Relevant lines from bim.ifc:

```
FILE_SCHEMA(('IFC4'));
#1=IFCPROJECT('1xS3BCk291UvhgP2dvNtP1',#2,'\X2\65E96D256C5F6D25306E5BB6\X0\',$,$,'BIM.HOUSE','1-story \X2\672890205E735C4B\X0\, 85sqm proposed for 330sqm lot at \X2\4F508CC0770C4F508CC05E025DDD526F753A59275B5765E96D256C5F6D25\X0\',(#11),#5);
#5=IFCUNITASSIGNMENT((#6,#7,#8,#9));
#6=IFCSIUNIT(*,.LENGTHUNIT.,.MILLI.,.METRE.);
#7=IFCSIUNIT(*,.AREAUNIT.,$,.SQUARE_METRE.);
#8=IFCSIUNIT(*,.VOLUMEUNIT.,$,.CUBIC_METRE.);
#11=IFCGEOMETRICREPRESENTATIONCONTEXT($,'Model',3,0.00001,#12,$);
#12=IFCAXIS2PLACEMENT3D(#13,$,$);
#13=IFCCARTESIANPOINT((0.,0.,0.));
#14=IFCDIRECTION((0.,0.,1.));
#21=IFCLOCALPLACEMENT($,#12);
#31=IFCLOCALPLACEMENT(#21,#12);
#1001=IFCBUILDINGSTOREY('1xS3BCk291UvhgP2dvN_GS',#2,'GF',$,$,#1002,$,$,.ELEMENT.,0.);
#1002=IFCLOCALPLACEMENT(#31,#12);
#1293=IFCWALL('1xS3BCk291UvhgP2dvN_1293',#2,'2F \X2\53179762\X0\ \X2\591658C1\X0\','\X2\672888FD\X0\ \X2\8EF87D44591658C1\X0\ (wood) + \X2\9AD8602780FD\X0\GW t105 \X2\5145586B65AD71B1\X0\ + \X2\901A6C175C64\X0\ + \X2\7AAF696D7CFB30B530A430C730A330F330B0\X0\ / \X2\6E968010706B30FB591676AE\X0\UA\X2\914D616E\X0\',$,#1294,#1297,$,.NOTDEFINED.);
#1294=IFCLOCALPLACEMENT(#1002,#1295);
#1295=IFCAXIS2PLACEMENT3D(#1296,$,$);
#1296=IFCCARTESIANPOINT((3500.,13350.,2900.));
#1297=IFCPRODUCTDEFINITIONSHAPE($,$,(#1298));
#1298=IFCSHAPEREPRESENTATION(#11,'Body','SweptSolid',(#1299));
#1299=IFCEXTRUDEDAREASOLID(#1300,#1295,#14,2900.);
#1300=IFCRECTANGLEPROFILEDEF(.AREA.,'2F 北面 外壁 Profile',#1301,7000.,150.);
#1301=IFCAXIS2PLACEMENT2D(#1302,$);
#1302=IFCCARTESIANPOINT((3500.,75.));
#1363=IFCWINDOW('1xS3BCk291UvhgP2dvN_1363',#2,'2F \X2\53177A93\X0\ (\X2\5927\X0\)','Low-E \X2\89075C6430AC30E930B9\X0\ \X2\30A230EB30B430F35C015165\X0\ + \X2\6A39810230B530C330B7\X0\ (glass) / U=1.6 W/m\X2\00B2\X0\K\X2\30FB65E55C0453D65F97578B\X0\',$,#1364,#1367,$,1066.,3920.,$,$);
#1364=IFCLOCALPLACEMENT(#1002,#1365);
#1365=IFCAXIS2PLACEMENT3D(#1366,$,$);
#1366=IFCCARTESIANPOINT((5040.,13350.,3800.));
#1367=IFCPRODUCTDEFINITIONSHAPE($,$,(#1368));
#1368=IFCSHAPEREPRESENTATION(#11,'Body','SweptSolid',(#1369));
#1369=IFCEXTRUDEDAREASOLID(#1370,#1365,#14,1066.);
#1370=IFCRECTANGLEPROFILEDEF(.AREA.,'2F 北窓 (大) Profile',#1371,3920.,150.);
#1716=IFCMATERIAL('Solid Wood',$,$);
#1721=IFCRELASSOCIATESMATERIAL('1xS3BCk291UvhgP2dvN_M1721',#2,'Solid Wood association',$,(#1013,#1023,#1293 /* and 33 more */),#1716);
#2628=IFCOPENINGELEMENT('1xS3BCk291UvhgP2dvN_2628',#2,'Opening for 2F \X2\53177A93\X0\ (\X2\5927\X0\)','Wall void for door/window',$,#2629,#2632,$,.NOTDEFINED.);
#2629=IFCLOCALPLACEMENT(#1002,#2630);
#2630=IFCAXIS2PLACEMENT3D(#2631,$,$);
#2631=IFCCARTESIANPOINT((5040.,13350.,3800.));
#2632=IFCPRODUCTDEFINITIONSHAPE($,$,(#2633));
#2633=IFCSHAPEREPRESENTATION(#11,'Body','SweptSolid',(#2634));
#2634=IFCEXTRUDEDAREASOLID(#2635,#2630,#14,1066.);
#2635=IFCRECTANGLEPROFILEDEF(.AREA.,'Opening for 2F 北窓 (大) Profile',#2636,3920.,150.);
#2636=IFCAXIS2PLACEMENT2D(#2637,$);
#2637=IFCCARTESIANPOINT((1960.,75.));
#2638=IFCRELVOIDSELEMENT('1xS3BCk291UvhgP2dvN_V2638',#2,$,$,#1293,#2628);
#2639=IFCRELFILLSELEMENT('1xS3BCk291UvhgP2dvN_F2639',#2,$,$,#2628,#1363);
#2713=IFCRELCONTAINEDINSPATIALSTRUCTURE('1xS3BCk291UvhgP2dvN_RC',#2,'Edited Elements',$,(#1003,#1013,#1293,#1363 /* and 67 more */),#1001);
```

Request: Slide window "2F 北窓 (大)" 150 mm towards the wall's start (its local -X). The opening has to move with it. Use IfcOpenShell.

```python
import ifcopenshell
import ifcopenshell.api.geometry
import ifcopenshell.util.placement
import ifcopenshell.util.unit

model = ifcopenshell.open("bim.ifc")
unit_scale = ifcopenshell.util.unit.calculate_unit_scale(model)

window = model.by_id(1363)
opening = window.FillsVoids[0].RelatingOpeningElement
wall = opening.VoidsElements[0].RelatingBuildingElement

wall_matrix = ifcopenshell.util.placement.get_local_placement(wall.ObjectPlacement)
shift = wall_matrix[:3, 0] * -0.15 / unit_scale
before = ifcopenshell.util.placement.get_local_placement(window.ObjectPlacement)[:3, 3].copy()

# The window is not placed relative to its opening, so move both.
for product in (opening, window):
    matrix = ifcopenshell.util.placement.get_local_placement(product.ObjectPlacement)
    matrix[:3, 3] += shift
    ifcopenshell.api.geometry.edit_object_placement(model, product=product, matrix=matrix, is_si=False)

after = ifcopenshell.util.placement.get_local_placement(window.ObjectPlacement)[:3, 3]
print("window moved by", (after - before).round(3) + 0.0)

model.write("bim-out.ifc")
```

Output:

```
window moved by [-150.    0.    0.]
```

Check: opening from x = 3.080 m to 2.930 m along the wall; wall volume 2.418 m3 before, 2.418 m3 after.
